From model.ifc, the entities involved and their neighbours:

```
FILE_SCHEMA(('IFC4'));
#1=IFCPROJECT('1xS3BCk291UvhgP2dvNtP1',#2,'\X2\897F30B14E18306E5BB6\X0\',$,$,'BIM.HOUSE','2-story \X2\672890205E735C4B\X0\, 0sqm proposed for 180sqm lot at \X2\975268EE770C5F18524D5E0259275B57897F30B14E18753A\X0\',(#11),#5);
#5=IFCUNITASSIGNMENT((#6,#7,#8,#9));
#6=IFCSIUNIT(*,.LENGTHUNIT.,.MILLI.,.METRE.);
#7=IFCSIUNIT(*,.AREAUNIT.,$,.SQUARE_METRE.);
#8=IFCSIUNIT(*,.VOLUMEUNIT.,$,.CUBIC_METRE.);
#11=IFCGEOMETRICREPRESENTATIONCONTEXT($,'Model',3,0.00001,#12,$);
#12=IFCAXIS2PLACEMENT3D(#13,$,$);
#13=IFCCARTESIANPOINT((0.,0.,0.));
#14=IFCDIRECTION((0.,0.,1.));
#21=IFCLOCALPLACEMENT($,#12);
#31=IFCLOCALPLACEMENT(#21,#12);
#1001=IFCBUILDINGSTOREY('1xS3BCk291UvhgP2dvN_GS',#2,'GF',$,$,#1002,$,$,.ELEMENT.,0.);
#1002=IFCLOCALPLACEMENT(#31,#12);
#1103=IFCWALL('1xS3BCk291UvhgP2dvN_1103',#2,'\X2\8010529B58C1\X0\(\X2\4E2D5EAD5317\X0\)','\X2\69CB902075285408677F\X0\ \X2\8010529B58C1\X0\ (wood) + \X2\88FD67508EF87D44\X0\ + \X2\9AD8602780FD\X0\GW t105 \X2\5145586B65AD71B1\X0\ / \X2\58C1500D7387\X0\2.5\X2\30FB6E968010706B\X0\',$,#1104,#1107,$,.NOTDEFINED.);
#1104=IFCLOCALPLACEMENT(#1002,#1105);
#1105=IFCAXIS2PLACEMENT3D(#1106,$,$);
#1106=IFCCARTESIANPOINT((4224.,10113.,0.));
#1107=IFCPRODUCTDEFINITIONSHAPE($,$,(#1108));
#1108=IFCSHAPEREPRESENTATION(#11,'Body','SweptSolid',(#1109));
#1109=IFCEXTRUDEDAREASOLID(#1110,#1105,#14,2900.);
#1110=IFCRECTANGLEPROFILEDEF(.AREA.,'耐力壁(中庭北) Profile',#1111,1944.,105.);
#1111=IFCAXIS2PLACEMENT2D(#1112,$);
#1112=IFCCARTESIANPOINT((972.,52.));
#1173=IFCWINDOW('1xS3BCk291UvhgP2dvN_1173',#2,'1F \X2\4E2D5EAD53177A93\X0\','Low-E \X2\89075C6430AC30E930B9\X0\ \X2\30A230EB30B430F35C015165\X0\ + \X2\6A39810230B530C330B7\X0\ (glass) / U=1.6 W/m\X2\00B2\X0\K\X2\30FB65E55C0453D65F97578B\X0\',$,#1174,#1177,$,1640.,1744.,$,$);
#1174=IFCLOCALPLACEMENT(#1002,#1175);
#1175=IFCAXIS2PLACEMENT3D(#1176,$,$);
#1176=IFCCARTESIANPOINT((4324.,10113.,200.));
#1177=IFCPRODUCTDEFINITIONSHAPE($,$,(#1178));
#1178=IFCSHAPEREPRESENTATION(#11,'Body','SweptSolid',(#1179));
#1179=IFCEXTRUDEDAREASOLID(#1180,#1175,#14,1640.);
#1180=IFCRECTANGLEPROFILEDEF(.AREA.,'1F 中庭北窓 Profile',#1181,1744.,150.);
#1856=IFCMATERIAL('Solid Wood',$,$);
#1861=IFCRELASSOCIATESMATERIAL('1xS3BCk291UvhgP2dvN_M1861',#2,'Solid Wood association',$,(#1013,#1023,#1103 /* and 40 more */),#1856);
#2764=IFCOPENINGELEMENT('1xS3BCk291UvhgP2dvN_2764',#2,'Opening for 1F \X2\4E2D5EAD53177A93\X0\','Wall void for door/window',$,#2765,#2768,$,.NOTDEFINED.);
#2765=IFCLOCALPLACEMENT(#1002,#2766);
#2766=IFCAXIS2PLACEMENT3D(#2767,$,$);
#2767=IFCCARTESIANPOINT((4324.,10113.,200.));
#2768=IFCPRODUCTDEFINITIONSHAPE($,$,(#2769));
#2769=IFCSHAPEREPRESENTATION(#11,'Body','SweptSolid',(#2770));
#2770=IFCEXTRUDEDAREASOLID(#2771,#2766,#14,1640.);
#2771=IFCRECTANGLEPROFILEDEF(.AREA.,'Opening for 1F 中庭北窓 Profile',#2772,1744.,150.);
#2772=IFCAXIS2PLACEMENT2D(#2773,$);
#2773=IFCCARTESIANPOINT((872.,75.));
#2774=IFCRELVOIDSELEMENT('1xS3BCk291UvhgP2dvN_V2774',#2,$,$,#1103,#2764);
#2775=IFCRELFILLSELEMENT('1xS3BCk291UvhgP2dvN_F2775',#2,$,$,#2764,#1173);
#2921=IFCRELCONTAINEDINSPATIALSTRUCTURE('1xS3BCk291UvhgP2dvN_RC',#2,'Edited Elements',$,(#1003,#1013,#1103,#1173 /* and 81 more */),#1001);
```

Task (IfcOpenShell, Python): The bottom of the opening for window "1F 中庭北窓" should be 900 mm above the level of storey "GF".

```python
import numpy as np
import ifcopenshell
import ifcopenshell.api.geometry
import ifcopenshell.geom
import ifcopenshell.util.element
import ifcopenshell.util.placement
import ifcopenshell.util.shape
import ifcopenshell.util.unit

model = ifcopenshell.open("model.ifc")
unit_scale = ifcopenshell.util.unit.calculate_unit_scale(model)

window = model.by_id(1173)
opening = window.FillsVoids[0].RelatingOpeningElement
storey = ifcopenshell.util.element.get_container(window, ifc_class="IfcBuildingStorey")
level = ifcopenshell.util.placement.get_local_placement(storey.ObjectPlacement)[2, 3]

# The opening's origin need not be at the sill, so measure its lowest point.
shape = ifcopenshell.geom.create_shape(ifcopenshell.geom.settings(), opening)
bottom = ifcopenshell.util.shape.get_shape_bottom_elevation(shape, shape.geometry) / unit_scale
dz = level + 0.9 / unit_scale - bottom

shift = np.array([0.0, 0.0, dz])
# The window is not placed relative to its opening, so move both.
for product in (opening, window):
    matrix = ifcopenshell.util.placement.get_local_placement(product.ObjectPlacement)
    matrix[:3, 3] += shift
    ifcopenshell.api.geometry.edit_object_placement(model, product=product, matrix=matrix, is_si=False)

print(f"moved by {dz * unit_scale:+.3f} m")

model.write("model_edited.ifc")
```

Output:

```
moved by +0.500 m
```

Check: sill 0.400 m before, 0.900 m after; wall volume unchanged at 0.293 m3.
